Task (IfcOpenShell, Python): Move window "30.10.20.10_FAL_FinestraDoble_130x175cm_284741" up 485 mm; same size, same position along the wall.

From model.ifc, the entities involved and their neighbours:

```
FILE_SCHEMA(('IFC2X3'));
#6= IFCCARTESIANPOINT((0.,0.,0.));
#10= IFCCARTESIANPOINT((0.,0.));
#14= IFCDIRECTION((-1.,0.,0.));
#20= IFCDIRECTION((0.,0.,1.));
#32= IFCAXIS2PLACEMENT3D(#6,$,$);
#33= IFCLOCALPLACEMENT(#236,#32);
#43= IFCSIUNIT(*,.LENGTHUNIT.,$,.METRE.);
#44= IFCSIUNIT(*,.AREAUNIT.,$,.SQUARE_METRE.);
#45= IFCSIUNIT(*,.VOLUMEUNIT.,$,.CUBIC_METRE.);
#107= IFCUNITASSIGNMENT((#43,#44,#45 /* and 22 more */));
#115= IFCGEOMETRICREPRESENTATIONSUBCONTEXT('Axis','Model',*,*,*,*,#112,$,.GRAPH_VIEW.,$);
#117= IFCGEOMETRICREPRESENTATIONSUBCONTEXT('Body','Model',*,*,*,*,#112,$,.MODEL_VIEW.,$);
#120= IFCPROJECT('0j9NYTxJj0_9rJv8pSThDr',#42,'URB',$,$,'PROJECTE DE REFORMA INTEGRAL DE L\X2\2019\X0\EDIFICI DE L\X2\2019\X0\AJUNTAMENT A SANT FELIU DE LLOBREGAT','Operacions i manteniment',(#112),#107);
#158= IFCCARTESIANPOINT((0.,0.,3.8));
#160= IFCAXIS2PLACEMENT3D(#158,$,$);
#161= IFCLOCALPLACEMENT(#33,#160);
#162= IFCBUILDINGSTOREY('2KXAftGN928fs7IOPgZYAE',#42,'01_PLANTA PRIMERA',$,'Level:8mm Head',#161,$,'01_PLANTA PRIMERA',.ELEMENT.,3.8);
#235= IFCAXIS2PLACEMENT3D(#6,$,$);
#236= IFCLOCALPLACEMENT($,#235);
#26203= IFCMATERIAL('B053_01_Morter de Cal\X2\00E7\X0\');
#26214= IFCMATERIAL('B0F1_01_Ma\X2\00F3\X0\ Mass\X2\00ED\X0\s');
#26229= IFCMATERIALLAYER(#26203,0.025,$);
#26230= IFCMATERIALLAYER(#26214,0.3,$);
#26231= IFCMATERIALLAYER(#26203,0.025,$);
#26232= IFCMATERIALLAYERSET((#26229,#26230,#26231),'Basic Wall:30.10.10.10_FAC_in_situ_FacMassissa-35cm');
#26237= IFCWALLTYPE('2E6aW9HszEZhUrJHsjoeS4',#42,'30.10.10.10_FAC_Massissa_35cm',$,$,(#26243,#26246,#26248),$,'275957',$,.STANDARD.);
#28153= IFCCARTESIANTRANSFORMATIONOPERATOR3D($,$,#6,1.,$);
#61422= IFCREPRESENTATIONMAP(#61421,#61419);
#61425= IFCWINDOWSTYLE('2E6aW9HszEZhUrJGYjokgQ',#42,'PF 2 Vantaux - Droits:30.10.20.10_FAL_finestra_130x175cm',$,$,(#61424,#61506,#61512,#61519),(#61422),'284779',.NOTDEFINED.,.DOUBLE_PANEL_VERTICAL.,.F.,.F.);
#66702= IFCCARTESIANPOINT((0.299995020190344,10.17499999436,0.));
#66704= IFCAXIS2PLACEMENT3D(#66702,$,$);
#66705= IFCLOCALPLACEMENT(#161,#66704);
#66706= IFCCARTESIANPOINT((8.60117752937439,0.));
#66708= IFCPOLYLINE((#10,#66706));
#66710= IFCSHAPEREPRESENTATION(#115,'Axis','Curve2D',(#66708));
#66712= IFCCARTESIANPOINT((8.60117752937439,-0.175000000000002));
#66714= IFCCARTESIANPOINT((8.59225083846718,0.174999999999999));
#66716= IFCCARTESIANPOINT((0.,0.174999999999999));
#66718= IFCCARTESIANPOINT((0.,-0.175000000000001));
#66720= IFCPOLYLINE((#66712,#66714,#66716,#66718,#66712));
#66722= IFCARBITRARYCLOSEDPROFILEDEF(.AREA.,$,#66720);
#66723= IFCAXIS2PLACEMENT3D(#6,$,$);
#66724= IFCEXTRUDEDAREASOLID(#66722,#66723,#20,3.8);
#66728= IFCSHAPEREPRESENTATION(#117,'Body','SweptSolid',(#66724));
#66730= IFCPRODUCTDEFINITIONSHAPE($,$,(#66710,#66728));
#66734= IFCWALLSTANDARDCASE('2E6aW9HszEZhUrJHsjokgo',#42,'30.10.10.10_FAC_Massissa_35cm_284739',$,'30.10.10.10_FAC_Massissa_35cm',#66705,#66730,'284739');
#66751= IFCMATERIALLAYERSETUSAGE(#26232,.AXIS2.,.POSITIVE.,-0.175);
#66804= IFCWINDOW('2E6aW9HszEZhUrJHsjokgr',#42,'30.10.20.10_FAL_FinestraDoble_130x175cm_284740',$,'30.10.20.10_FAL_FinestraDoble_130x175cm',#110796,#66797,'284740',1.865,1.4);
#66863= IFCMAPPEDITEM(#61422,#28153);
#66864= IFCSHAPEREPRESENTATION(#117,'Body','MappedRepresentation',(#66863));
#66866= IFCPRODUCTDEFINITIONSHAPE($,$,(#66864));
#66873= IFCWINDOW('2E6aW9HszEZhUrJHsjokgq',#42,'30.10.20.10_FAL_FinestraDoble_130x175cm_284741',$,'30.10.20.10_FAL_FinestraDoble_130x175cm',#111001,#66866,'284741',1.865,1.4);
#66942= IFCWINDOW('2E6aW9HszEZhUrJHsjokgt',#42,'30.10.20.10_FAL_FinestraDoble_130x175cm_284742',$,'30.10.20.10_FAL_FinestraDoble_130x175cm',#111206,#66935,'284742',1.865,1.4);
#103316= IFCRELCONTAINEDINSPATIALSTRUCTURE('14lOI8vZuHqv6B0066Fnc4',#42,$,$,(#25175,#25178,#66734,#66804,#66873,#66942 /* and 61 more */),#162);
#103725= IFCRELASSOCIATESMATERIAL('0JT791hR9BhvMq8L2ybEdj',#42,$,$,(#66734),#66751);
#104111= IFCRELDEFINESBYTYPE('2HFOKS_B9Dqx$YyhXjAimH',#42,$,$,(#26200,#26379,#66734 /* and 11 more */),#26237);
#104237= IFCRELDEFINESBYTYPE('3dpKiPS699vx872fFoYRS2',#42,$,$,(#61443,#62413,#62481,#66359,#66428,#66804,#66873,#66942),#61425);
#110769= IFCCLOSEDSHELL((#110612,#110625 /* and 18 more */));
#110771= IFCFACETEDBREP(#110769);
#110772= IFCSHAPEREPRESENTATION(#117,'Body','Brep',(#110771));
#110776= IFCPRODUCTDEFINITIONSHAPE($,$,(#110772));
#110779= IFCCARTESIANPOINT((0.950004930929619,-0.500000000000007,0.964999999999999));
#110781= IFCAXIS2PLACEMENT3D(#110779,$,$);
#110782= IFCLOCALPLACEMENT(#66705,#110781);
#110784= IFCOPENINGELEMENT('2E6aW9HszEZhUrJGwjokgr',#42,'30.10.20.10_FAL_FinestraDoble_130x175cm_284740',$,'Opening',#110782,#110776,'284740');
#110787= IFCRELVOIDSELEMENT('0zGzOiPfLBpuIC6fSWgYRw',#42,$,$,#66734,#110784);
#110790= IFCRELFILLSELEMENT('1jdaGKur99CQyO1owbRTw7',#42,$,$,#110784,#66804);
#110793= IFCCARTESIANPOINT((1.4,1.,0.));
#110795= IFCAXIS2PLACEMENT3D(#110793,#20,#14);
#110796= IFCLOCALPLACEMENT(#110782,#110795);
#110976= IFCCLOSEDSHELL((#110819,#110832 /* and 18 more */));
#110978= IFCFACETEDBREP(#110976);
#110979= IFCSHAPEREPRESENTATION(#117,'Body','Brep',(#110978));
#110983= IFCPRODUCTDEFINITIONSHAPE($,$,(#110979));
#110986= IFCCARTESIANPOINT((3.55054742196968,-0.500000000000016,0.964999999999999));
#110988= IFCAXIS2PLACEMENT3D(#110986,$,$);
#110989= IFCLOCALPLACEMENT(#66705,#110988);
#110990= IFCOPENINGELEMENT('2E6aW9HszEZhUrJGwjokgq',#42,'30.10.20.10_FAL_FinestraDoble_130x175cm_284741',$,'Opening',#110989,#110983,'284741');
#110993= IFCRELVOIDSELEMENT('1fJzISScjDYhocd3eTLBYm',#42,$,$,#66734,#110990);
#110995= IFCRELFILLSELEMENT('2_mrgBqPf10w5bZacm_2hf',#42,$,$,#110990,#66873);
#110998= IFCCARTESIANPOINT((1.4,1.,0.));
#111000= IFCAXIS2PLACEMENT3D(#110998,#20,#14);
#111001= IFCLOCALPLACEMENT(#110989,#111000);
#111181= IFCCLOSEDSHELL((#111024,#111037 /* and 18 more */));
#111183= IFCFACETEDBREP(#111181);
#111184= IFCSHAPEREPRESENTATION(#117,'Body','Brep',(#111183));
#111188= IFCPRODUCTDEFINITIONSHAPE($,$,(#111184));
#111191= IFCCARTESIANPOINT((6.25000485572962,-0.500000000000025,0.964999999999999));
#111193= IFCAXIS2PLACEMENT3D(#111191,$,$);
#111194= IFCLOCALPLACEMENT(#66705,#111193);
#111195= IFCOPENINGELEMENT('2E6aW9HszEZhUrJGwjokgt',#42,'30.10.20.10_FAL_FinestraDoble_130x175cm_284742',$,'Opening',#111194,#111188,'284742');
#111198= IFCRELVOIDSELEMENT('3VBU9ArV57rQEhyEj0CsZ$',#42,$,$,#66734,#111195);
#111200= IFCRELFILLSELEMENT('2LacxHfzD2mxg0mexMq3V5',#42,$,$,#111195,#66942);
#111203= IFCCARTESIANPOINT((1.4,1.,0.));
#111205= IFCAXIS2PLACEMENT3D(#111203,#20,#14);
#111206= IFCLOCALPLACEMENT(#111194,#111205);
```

```python
import numpy as np
import ifcopenshell
import ifcopenshell.api.geometry
import ifcopenshell.util.placement
import ifcopenshell.util.unit

model = ifcopenshell.open("model.ifc")
unit_scale = ifcopenshell.util.unit.calculate_unit_scale(model)

window = model.by_id(66873)
opening = window.FillsVoids[0].RelatingOpeningElement
dz = 0.485 / unit_scale

shift = np.array([0.0, 0.0, dz])
# The window is placed relative to its opening, so it follows when the opening moves.
matrix = ifcopenshell.util.placement.get_local_placement(opening.ObjectPlacement)
matrix[:3, 3] += shift
ifcopenshell.api.geometry.edit_object_placement(
    model, product=opening, matrix=matrix, is_si=False, should_transform_children=True
)

print(f"moved by {dz * unit_scale:+.3f} m")

model.write("model_rev.ifc")
```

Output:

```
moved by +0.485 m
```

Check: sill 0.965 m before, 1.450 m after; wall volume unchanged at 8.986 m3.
